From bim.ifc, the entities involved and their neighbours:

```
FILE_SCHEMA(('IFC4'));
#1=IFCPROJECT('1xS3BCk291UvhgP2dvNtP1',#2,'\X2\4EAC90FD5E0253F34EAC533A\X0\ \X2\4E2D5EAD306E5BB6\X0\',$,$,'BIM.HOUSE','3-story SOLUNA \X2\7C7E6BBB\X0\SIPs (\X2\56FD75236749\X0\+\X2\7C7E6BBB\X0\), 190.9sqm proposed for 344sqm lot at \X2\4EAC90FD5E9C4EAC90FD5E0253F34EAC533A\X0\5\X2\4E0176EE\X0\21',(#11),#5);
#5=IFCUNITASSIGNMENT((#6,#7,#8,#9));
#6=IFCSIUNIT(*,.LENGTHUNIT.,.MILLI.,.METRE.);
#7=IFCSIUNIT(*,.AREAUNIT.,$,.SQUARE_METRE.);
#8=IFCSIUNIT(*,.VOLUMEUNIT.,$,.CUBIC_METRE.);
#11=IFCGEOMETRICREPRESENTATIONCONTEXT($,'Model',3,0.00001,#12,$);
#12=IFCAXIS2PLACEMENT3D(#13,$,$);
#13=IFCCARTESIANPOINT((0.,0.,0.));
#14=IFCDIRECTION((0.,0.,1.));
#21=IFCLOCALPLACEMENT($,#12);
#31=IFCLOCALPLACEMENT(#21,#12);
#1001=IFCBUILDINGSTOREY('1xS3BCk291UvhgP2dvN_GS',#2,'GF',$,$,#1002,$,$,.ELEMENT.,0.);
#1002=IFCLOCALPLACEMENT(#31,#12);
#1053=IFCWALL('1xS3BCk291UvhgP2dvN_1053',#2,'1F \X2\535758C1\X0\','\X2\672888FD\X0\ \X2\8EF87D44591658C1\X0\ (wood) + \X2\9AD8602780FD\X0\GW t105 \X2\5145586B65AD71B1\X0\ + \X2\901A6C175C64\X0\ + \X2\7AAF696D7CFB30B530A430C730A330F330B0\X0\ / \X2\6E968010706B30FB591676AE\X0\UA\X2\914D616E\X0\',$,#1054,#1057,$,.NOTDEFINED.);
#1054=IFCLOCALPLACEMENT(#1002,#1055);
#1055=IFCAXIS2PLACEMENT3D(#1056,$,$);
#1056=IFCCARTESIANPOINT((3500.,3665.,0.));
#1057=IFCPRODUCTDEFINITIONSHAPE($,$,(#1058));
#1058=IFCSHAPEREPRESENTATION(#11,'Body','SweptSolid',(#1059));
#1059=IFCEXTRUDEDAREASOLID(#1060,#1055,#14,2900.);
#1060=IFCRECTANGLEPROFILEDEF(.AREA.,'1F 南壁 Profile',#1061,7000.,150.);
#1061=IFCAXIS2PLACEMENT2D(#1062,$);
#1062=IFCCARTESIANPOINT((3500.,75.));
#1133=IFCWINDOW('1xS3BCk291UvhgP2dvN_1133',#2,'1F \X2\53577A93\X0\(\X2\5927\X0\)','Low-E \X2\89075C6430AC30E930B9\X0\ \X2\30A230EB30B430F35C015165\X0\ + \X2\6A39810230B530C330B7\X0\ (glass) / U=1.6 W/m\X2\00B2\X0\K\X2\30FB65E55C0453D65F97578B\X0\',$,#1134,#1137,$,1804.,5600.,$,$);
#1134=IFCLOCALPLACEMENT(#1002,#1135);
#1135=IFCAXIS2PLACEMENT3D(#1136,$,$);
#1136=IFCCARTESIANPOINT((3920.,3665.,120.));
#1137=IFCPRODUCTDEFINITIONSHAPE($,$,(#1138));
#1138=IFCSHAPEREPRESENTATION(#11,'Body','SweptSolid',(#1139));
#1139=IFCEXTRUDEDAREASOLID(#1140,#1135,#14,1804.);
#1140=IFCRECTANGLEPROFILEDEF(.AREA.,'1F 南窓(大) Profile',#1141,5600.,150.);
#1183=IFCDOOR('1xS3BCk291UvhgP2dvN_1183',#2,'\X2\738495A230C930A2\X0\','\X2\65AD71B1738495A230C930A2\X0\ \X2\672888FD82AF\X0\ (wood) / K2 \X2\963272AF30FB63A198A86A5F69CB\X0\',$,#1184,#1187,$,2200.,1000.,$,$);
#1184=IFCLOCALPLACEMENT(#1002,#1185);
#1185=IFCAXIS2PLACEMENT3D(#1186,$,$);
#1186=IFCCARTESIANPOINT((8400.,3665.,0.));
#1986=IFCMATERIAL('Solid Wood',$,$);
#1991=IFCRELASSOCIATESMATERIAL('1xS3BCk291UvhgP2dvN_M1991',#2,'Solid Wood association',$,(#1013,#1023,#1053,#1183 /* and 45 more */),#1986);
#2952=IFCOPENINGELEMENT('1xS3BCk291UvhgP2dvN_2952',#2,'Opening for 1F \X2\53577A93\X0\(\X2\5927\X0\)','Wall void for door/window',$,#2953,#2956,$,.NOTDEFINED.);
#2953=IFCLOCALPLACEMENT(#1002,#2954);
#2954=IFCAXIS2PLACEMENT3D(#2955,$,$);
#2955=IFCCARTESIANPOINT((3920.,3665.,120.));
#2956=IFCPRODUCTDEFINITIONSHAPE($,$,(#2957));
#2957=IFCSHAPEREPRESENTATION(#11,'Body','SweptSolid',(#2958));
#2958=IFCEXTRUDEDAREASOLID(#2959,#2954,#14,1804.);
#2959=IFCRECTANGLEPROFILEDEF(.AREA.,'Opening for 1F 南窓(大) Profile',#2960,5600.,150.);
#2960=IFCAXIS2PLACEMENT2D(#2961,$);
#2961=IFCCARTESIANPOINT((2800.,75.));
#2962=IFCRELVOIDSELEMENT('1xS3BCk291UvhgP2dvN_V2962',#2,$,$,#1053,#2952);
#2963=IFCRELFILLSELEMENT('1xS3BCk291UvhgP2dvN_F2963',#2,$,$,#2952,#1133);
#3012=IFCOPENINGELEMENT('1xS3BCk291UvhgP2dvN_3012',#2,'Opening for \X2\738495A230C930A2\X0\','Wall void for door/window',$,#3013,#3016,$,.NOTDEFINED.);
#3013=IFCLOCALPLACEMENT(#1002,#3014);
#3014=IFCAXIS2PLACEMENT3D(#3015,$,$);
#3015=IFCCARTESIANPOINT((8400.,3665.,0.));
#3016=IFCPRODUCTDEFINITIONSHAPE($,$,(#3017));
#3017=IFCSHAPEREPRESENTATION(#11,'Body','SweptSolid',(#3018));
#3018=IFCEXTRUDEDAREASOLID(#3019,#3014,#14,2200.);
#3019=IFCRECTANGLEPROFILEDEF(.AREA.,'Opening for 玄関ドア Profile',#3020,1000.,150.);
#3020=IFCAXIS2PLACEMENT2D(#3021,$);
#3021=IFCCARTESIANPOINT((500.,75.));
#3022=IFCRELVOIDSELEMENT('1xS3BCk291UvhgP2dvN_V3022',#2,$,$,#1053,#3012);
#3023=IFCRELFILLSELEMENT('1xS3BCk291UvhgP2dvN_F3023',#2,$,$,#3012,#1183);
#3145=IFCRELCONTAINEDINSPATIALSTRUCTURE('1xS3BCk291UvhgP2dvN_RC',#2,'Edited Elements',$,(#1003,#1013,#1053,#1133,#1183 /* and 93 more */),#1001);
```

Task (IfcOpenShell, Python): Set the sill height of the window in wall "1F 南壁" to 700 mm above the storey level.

```python
import numpy as np
import ifcopenshell
import ifcopenshell.api.geometry
import ifcopenshell.geom
import ifcopenshell.util.element
import ifcopenshell.util.placement
import ifcopenshell.util.shape
import ifcopenshell.util.unit

model = ifcopenshell.open("bim.ifc")
unit_scale = ifcopenshell.util.unit.calculate_unit_scale(model)

window = model.by_guid("1xS3BCk291UvhgP2dvN_1133")
opening = window.FillsVoids[0].RelatingOpeningElement
storey = ifcopenshell.util.element.get_container(window, ifc_class="IfcBuildingStorey")
level = ifcopenshell.util.placement.get_local_placement(storey.ObjectPlacement)[2, 3]

# The opening's origin need not be at the sill, so measure its lowest point.
shape = ifcopenshell.geom.create_shape(ifcopenshell.geom.settings(), opening)
bottom = ifcopenshell.util.shape.get_shape_bottom_elevation(shape, shape.geometry) / unit_scale
dz = level + 0.7 / unit_scale - bottom

shift = np.array([0.0, 0.0, dz])
# The window is not placed relative to its opening, so move both.
for product in (opening, window):
    matrix = ifcopenshell.util.placement.get_local_placement(product.ObjectPlacement)
    matrix[:3, 3] += shift
    ifcopenshell.api.geometry.edit_object_placement(model, product=product, matrix=matrix, is_si=False)

print(f"moved by {dz * unit_scale:+.3f} m")

model.write("bim_rev.ifc")
```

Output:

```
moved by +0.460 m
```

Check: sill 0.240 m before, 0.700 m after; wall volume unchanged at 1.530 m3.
